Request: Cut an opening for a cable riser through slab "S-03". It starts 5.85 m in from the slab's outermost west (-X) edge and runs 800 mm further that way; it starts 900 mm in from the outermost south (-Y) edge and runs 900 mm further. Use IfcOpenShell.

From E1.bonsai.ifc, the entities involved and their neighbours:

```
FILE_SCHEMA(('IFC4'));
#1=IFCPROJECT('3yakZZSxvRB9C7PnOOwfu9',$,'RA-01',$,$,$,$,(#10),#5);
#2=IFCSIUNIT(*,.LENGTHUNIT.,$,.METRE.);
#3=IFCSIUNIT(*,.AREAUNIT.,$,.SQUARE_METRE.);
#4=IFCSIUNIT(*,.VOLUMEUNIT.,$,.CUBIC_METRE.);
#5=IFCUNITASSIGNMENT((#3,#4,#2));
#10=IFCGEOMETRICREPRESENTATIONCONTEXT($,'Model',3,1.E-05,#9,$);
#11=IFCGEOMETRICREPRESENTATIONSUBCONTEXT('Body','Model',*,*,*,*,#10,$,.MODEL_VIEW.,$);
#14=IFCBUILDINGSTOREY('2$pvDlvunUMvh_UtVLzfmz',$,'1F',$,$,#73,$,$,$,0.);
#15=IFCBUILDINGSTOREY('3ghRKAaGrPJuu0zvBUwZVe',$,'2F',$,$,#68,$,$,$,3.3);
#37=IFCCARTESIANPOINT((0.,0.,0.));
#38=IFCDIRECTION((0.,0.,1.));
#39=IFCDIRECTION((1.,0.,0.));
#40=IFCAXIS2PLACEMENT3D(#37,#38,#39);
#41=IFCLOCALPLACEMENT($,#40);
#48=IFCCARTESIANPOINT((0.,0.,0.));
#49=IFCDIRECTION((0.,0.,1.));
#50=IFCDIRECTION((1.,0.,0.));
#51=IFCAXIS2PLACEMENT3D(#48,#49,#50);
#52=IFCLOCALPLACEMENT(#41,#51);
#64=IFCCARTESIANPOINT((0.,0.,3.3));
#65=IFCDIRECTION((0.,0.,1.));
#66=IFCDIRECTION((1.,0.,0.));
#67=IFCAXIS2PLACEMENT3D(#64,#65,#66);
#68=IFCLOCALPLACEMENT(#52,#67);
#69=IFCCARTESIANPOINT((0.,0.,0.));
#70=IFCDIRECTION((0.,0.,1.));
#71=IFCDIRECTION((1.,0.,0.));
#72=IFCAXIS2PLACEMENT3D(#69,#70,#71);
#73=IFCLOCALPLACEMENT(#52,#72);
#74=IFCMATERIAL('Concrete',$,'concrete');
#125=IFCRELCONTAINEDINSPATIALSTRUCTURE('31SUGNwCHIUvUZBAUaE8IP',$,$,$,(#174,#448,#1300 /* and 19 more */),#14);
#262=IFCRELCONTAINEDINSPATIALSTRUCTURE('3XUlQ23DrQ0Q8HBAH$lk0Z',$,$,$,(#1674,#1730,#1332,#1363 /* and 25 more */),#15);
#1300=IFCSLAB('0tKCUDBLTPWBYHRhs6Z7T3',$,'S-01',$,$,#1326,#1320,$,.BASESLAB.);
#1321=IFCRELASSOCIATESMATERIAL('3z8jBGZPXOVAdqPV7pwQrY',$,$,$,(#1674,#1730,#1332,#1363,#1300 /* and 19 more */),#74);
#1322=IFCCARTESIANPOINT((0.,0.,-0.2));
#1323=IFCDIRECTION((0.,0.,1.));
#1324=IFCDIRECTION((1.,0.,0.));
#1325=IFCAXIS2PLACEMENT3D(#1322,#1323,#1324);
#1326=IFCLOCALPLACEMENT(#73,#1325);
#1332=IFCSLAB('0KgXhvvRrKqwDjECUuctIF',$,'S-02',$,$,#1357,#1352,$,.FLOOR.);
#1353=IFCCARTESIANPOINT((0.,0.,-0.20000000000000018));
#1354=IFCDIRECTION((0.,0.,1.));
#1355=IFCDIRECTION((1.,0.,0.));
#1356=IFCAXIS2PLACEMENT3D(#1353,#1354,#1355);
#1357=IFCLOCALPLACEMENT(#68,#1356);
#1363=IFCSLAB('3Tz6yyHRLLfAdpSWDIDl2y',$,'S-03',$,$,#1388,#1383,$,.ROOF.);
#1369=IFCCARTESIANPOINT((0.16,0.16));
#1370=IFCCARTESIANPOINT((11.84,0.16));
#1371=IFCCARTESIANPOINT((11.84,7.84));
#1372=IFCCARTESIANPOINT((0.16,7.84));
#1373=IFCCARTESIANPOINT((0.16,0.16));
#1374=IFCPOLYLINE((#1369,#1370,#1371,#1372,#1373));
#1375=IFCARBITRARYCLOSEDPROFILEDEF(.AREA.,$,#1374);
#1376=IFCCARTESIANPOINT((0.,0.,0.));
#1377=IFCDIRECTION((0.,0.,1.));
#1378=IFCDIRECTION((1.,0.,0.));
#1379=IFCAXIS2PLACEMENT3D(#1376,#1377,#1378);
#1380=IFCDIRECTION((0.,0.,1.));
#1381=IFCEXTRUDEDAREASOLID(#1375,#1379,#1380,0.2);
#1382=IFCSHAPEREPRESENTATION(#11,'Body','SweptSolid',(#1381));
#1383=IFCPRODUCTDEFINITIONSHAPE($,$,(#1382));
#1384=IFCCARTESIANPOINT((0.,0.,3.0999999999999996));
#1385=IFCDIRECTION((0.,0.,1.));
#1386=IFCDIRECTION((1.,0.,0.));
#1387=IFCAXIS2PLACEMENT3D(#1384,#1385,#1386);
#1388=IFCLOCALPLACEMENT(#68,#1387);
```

```python
import numpy as np
import ifcopenshell
import ifcopenshell.api.feature
import ifcopenshell.api.geometry
import ifcopenshell.api.root
import ifcopenshell.geom
import ifcopenshell.util.placement
import ifcopenshell.util.representation
import ifcopenshell.util.shape
import ifcopenshell.util.unit

model = ifcopenshell.open("E1.bonsai.ifc")
unit_scale = ifcopenshell.util.unit.calculate_unit_scale(model)
settings = ifcopenshell.geom.settings()


def volume(element):
    """Net volume in cubic metres, openings subtracted."""
    shape = ifcopenshell.geom.create_shape(settings, element)
    return ifcopenshell.util.shape.get_volume(shape.geometry)


slab = model.by_guid("3Tz6yyHRLLfAdpSWDIDl2y")
before = volume(slab)

# Extent in the slab's own axes, in metres. The edges named are its -X and -Y sides.
slab_shape = ifcopenshell.geom.create_shape(settings, slab)
vertices = ifcopenshell.util.shape.get_vertices(slab_shape.geometry)
x_min, y_min, bottom = vertices.min(axis=0)
top = vertices[:, 2].max()

opening = ifcopenshell.api.root.create_entity(model, ifc_class="IfcOpeningElement", name="Cable riser opening", predefined_type="OPENING")
context = ifcopenshell.util.representation.get_context(model, "Model", "Body", "MODEL_VIEW")
width, depth = 0.8, 0.9
outline = [(0.0, 0.0), (width, 0.0), (width, depth), (0.0, depth), (0.0, 0.0)]
# Overshoot both faces by 50 mm so the cut is clean.
shape = ifcopenshell.api.geometry.add_slab_representation(
    model, context=context, depth=top - bottom + 0.1, polyline=outline
)
ifcopenshell.api.geometry.assign_representation(model, product=opening, representation=shape)

matrix = ifcopenshell.util.placement.get_local_placement(slab.ObjectPlacement)
matrix[:, 3] = matrix @ np.append(np.array([x_min + 5.85, y_min + 0.9, bottom - 0.05]) / unit_scale, 1.0)
ifcopenshell.api.geometry.edit_object_placement(model, product=opening, matrix=matrix, is_si=False)
ifcopenshell.api.feature.add_feature(model, feature=opening, element=slab)

after = volume(slab)

print(f"slab volume {before:.3f} -> {after:.3f} m3")

model.write("E1.bonsai_v2.ifc")
```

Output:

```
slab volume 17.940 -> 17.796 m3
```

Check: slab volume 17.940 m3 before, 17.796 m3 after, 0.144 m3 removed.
